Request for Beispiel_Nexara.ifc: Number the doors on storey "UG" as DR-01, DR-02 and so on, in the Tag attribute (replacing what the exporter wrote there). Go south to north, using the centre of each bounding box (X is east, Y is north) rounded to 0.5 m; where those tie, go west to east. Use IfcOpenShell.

First a look at what the model holds.

```python
import ifcopenshell
import ifcopenshell.util.element
import ifcopenshell.util.placement

model = ifcopenshell.open("Beispiel_Nexara.ifc")
print(model.schema)
storey = next(s for s in model.by_type("IfcBuildingStorey") if s.Name == "UG")
doors = [e for e in ifcopenshell.util.element.get_decomposition(storey) if e.is_a("IfcDoor")]
for e in sorted(doors, key=lambda e: e.id()):
    origin = ifcopenshell.util.placement.get_local_placement(e.ObjectPlacement)[:3, 3]
    print(e.id(), e.Tag, e.Name, origin.round(2) + 0.0, sep=" | ")
```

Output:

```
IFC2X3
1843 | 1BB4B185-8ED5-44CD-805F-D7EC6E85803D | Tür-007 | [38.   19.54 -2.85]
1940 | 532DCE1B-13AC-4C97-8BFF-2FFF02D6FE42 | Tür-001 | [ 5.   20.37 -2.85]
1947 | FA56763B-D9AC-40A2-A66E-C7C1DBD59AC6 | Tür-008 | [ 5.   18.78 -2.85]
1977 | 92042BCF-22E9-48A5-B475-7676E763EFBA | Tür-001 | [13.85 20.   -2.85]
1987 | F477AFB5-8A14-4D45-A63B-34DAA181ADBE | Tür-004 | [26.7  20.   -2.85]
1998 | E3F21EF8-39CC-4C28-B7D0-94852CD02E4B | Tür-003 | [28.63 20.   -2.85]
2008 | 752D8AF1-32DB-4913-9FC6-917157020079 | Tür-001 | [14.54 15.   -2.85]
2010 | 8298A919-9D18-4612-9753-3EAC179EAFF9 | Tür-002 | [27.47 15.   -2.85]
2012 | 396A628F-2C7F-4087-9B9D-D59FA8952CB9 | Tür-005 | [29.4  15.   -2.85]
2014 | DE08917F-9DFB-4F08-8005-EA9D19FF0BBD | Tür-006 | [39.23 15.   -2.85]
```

```python
import ifcopenshell
import ifcopenshell.geom
import ifcopenshell.util.element
import ifcopenshell.util.shape

model = ifcopenshell.open("Beispiel_Nexara.ifc")
settings = ifcopenshell.geom.settings()
settings.set("use-world-coords", True)


def centre(element):
    shape = ifcopenshell.geom.create_shape(settings, element)
    return ifcopenshell.util.shape.get_bbox_centroid(shape.geometry)


storey = next(s for s in model.by_type("IfcBuildingStorey") if s.Name == "UG")
doors = [e for e in ifcopenshell.util.element.get_decomposition(storey) if e.is_a("IfcDoor")]

# Insertion points can sit at a corner or the storey origin, so sort by the geometry (in metres).
centres = {e: centre(e) for e in doors}
doors.sort(key=lambda e: (round(centres[e][1] / 0.5), centres[e][0]))

for i, e in enumerate(doors, start=1):
    number = f"DR-{i:02d}"
    e.Tag = number
    print(e.id(), number)

model.write("Beispiel_Nexara-out.ifc")
```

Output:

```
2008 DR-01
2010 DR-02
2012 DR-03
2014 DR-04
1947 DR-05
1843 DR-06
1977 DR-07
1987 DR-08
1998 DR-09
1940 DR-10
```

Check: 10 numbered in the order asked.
